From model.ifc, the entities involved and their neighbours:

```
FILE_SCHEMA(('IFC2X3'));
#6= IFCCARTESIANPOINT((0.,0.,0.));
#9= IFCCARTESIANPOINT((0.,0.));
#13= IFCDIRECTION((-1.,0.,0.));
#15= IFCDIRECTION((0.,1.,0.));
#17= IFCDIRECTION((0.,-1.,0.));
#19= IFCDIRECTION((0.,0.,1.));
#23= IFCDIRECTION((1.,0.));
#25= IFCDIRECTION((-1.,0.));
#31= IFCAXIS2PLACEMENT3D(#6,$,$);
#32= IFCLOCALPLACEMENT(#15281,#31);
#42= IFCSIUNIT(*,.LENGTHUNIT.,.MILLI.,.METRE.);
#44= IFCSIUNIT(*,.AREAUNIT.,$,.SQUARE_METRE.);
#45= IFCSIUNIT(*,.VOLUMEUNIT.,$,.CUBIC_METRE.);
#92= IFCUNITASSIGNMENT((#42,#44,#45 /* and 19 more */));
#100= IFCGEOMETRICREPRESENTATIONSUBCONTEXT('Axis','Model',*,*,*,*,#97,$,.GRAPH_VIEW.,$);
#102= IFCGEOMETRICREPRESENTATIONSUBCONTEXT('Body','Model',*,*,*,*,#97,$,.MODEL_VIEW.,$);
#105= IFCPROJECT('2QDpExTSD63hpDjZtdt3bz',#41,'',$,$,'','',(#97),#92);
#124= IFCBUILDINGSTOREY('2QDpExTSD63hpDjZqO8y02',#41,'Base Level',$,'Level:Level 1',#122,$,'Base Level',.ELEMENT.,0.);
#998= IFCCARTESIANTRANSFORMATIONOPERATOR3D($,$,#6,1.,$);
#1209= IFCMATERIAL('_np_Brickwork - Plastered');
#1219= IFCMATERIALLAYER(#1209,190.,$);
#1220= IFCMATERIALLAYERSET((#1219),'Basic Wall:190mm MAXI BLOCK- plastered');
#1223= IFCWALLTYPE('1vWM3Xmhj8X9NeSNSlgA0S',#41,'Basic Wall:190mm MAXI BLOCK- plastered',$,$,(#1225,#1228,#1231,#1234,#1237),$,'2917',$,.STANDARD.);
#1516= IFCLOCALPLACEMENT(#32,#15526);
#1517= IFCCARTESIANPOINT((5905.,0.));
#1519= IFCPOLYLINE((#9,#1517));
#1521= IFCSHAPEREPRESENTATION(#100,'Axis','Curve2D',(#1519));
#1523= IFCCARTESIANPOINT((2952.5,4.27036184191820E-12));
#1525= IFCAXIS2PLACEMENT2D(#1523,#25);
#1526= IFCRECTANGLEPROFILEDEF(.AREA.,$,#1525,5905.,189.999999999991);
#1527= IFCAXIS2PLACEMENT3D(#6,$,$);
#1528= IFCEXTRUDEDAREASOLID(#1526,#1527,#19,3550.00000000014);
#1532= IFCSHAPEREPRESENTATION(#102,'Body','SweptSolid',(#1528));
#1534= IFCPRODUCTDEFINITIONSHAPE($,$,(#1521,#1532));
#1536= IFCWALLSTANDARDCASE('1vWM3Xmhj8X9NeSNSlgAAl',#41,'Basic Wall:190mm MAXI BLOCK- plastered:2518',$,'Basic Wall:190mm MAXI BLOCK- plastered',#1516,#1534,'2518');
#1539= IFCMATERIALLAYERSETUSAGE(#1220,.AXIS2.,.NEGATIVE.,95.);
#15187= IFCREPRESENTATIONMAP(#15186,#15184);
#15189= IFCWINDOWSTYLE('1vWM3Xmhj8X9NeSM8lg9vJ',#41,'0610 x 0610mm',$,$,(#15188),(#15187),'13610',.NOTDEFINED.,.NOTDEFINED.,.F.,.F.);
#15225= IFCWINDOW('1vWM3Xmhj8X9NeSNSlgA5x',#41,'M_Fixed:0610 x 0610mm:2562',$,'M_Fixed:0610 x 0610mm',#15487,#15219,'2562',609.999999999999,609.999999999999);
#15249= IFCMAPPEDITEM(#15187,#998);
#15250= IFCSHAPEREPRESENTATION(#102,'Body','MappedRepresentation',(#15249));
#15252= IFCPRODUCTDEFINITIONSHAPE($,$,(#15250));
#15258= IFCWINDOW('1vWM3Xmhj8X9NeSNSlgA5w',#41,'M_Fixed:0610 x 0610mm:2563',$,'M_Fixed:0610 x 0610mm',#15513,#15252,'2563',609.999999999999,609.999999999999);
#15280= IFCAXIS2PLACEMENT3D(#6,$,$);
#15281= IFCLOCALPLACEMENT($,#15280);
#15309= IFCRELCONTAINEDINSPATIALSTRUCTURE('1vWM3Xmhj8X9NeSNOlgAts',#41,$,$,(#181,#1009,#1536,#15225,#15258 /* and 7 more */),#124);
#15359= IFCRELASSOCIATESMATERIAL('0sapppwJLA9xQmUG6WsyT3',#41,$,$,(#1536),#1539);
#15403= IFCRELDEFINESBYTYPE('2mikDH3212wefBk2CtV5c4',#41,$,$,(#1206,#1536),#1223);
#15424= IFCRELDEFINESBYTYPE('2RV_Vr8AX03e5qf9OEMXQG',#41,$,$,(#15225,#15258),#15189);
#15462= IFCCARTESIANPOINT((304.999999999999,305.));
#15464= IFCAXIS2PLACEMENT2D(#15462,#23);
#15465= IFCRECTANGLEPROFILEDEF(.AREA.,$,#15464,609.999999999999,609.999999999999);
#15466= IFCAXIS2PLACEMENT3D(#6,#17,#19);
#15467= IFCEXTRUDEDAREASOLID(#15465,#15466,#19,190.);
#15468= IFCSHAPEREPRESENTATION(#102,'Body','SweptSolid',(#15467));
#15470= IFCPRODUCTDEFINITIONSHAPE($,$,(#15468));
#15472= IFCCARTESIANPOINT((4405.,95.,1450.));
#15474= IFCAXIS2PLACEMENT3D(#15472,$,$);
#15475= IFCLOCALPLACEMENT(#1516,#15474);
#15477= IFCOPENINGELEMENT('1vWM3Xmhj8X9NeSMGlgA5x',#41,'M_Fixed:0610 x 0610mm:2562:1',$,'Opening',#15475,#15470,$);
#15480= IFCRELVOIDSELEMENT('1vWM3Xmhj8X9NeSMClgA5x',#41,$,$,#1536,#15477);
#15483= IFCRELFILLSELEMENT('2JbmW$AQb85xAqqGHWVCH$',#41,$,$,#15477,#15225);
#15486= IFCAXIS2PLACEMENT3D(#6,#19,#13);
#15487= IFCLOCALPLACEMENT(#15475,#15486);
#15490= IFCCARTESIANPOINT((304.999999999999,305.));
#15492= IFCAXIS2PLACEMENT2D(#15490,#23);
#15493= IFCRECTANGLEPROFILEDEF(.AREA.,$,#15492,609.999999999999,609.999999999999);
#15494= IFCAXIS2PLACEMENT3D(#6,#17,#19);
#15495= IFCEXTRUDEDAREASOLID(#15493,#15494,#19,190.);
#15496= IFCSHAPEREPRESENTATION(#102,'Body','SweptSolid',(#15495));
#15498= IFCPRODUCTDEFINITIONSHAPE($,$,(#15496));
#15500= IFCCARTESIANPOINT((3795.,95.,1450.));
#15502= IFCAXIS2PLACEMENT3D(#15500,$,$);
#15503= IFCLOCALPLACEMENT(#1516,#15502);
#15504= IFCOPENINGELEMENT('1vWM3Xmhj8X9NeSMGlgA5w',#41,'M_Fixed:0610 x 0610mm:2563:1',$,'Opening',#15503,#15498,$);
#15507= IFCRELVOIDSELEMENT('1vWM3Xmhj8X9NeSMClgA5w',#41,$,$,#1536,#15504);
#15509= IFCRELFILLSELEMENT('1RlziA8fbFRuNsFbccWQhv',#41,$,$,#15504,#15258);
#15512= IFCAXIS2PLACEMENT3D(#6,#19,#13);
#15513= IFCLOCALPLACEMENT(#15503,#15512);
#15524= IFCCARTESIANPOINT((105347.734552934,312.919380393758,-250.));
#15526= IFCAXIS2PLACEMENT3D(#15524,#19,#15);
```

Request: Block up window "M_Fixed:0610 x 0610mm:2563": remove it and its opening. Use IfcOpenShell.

```python
import ifcopenshell
import ifcopenshell.api.feature
import ifcopenshell.api.root
import ifcopenshell.geom
import ifcopenshell.util.shape

model = ifcopenshell.open("model.ifc")
settings = ifcopenshell.geom.settings()


def volume(element):
    """Net volume in cubic metres, openings subtracted."""
    shape = ifcopenshell.geom.create_shape(settings, element)
    return ifcopenshell.util.shape.get_volume(shape.geometry)


window = model.by_guid("1vWM3Xmhj8X9NeSNSlgA5w")
opening = window.FillsVoids[0].RelatingOpeningElement
wall = opening.VoidsElements[0].RelatingBuildingElement
before = volume(wall)

ifcopenshell.api.root.remove_product(model, product=window)
ifcopenshell.api.feature.remove_feature(model, feature=opening)

after = volume(wall)

print(f"wall volume {before:.3f} -> {after:.3f} m3")

model.write("model-out.ifc")
```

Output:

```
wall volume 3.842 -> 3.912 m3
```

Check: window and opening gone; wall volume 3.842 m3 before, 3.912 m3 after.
